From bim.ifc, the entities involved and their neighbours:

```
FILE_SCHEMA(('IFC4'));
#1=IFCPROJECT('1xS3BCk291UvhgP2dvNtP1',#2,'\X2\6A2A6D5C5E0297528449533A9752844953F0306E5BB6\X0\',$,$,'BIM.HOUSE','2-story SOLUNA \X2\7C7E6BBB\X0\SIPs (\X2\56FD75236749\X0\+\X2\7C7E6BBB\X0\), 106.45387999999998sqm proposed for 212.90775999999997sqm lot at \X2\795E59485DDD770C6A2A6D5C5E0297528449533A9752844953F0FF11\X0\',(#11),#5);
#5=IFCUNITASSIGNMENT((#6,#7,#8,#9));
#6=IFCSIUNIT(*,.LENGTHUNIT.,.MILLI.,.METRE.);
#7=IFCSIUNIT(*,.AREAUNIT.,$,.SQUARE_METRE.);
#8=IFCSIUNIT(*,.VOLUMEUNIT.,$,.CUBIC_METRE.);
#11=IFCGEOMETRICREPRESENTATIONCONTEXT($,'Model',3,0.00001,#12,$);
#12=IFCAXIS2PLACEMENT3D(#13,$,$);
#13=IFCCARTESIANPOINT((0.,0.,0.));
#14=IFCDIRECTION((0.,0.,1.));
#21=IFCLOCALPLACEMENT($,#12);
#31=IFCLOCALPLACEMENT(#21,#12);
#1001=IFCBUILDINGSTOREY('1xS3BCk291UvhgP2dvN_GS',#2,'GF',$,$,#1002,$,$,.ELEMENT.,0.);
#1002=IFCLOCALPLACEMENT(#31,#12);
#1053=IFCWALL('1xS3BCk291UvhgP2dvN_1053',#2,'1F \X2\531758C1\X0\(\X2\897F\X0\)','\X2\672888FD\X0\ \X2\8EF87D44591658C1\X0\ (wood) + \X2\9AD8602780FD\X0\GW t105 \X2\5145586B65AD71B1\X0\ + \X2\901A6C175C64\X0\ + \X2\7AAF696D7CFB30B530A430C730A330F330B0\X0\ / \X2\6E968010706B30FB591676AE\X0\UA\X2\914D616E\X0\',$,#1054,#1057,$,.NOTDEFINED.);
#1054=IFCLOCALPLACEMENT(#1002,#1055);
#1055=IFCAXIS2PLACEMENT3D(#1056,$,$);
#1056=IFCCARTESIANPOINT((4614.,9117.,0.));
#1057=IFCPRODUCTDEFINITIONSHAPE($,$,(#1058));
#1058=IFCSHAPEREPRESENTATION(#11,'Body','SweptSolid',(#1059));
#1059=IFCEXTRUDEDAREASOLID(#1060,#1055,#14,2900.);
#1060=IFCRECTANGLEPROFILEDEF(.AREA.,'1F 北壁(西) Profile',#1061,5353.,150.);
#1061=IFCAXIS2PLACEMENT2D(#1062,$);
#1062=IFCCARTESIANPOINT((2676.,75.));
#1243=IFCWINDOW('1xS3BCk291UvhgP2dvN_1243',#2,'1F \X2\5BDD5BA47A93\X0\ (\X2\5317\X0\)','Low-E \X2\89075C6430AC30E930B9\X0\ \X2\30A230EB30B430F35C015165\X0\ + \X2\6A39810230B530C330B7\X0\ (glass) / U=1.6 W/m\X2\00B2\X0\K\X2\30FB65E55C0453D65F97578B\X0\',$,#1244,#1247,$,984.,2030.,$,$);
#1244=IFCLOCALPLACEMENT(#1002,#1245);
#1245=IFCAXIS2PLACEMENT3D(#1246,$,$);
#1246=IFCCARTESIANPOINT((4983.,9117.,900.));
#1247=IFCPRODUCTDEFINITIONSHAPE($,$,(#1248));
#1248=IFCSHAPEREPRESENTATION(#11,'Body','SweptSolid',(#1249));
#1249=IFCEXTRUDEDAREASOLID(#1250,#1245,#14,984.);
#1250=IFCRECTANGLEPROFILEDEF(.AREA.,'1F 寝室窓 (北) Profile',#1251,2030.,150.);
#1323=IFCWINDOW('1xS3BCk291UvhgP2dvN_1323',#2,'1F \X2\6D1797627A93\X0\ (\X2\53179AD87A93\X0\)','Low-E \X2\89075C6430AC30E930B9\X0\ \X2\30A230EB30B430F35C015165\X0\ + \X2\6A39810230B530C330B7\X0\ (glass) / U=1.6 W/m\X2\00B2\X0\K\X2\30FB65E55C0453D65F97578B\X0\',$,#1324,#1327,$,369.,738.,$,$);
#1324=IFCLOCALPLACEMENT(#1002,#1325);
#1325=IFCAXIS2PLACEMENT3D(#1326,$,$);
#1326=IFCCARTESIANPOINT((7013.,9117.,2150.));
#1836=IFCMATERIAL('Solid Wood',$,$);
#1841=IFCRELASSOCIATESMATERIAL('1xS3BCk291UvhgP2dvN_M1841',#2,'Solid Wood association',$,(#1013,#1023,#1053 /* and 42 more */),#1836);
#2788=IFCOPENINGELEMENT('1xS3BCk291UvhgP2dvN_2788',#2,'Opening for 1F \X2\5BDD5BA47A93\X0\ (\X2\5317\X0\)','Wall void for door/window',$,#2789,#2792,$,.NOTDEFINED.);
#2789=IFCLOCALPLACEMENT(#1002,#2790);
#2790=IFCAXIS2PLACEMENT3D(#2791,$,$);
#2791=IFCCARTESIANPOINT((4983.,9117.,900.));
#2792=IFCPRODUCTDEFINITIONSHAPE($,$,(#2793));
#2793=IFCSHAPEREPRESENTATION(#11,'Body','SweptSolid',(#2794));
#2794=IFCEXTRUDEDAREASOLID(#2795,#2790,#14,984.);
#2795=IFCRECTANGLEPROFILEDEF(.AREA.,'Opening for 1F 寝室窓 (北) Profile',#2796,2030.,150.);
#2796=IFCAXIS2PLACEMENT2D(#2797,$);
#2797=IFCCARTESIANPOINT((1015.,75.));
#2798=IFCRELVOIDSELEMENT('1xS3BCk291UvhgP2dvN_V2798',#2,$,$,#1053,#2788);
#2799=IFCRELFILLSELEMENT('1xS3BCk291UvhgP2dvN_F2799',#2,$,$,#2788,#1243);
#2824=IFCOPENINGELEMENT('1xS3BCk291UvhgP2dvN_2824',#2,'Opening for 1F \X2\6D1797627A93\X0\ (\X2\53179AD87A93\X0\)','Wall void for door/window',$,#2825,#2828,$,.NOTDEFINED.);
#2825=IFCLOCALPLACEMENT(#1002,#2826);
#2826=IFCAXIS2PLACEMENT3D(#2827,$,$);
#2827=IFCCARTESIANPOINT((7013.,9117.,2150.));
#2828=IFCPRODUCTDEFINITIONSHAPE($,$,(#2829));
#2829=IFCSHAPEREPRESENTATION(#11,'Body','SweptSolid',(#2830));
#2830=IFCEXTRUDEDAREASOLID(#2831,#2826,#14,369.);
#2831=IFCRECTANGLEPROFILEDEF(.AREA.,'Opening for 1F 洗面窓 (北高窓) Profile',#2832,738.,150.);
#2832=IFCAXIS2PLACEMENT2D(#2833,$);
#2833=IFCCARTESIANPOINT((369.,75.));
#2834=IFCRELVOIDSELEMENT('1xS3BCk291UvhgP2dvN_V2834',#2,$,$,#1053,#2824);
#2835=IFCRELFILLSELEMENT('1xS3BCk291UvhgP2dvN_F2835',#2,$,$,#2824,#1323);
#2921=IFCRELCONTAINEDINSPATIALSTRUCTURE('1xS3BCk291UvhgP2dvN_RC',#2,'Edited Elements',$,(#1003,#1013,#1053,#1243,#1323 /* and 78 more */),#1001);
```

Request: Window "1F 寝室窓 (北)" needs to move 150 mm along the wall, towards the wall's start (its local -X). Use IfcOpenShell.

```python
import ifcopenshell
import ifcopenshell.api.geometry
import ifcopenshell.util.placement
import ifcopenshell.util.unit

model = ifcopenshell.open("bim.ifc")
unit_scale = ifcopenshell.util.unit.calculate_unit_scale(model)

window = model.by_guid("1xS3BCk291UvhgP2dvN_1243")
opening = window.FillsVoids[0].RelatingOpeningElement
wall = opening.VoidsElements[0].RelatingBuildingElement

wall_matrix = ifcopenshell.util.placement.get_local_placement(wall.ObjectPlacement)
shift = wall_matrix[:3, 0] * -0.15 / unit_scale
before = ifcopenshell.util.placement.get_local_placement(window.ObjectPlacement)[:3, 3].copy()

# The window is not placed relative to its opening, so move both.
for product in (opening, window):
    matrix = ifcopenshell.util.placement.get_local_placement(product.ObjectPlacement)
    matrix[:3, 3] += shift
    ifcopenshell.api.geometry.edit_object_placement(model, product=product, matrix=matrix, is_si=False)

after = ifcopenshell.util.placement.get_local_placement(window.ObjectPlacement)[:3, 3]
print("window moved by", (after - before).round(3) + 0.0)

model.write("bim_rev.ifc")
```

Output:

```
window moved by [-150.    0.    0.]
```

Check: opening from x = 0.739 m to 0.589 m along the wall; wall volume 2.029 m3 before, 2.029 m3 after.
